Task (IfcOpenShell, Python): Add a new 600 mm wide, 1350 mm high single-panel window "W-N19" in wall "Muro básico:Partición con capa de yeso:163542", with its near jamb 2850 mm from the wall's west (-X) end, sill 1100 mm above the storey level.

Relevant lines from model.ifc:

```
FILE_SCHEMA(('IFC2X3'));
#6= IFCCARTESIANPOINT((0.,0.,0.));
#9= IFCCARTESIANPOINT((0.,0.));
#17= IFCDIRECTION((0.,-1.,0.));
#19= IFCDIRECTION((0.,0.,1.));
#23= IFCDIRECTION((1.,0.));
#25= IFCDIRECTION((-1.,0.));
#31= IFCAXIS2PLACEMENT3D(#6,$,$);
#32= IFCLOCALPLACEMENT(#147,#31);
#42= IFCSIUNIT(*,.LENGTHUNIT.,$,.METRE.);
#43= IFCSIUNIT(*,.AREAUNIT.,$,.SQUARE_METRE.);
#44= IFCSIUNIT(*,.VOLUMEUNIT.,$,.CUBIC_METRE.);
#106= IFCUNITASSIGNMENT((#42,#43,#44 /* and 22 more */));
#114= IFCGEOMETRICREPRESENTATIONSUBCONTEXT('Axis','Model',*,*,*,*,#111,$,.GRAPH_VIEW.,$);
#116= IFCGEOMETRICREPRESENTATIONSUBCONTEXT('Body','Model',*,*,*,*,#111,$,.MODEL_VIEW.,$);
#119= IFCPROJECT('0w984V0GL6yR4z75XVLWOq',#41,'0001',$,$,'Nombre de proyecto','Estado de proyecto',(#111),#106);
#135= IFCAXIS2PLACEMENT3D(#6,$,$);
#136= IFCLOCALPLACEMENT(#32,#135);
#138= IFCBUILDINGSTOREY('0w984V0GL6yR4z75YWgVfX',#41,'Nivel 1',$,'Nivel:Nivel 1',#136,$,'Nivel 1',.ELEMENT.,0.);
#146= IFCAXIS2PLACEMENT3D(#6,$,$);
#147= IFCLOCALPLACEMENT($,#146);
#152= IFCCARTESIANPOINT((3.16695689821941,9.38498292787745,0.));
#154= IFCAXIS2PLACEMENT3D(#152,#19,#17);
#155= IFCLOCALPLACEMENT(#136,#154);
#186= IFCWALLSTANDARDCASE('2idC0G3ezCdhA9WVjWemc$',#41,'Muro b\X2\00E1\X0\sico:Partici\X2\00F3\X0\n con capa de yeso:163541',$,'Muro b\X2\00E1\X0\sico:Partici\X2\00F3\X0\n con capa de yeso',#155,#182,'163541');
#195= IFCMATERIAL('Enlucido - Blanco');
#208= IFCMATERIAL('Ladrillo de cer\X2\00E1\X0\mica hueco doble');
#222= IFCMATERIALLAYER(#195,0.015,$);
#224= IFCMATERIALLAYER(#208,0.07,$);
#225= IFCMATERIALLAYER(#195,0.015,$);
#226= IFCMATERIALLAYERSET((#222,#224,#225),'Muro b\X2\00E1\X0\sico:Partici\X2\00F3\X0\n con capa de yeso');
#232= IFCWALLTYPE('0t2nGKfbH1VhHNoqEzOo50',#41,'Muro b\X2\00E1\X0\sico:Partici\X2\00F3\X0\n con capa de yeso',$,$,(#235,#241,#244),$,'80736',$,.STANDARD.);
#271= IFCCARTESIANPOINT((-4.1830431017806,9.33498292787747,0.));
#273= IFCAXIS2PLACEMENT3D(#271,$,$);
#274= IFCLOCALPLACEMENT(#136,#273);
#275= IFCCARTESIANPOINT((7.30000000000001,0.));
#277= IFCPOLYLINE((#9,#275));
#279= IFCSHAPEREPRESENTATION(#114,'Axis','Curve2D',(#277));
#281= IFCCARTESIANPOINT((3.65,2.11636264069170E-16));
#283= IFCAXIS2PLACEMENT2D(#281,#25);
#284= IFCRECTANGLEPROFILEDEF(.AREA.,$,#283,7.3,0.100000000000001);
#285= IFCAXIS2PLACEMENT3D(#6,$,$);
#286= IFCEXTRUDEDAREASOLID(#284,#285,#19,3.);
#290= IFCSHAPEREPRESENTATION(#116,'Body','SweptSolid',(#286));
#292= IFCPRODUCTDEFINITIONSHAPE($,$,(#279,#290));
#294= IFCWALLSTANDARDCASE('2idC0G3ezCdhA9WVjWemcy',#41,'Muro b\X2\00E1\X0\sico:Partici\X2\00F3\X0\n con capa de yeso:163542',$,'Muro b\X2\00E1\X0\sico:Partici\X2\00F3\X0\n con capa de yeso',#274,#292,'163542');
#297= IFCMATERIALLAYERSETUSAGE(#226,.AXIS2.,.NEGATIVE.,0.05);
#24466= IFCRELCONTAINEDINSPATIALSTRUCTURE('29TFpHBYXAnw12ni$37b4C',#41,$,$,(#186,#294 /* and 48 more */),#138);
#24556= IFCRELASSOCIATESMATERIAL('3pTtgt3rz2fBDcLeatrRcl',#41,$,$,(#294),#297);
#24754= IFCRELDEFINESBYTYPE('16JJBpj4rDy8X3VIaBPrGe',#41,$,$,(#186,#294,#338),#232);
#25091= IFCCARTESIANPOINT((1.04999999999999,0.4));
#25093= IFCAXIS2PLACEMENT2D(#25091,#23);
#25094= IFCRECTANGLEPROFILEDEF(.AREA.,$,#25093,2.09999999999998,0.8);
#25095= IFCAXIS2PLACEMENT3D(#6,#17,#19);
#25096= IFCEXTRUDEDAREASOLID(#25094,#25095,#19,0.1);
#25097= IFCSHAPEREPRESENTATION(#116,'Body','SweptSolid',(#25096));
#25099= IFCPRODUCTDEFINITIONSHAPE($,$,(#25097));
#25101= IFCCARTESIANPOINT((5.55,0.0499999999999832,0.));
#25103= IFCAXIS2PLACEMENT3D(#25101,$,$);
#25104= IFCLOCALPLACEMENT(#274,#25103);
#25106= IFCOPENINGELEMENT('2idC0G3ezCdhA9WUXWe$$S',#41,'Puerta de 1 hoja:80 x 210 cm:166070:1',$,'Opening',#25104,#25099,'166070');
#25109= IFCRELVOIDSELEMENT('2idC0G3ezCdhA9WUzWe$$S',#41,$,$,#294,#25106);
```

```python
import numpy as np
import ifcopenshell
import ifcopenshell.api.feature
import ifcopenshell.api.geometry
import ifcopenshell.api.root
import ifcopenshell.api.spatial
import ifcopenshell.api.type
import ifcopenshell.geom
import ifcopenshell.util.element
import ifcopenshell.util.placement
import ifcopenshell.util.representation
import ifcopenshell.util.shape
import ifcopenshell.util.unit

model = ifcopenshell.open("model.ifc")
unit_scale = ifcopenshell.util.unit.calculate_unit_scale(model)
settings = ifcopenshell.geom.settings()


def volume(element):
    """Net volume in cubic metres, openings subtracted."""
    shape = ifcopenshell.geom.create_shape(settings, element)
    return ifcopenshell.util.shape.get_volume(shape.geometry)


wall = model.by_id(294)
storey = ifcopenshell.util.element.get_container(wall, ifc_class="IfcBuildingStorey")
context = ifcopenshell.util.representation.get_context(model, "Model", "Body", "MODEL_VIEW")
before = volume(wall)

width, height, from_end, sill = 0.6, 1.35, 2.85, 1.1  # metres

# The wall runs along its own X axis, and the end named is its -X end.
wall_shape = ifcopenshell.geom.create_shape(settings, wall)
x, y, z = ifcopenshell.util.shape.get_vertices(wall_shape.geometry).T
start = x.min() + from_end
face, thickness = float(y.min()), float(y.max() - y.min())
wall_matrix = ifcopenshell.util.placement.get_local_placement(wall.ObjectPlacement)
level = ifcopenshell.util.placement.get_local_placement(storey.ObjectPlacement)[2, 3]


def in_wall(x, y):
    """Placement at x, y metres in the wall's axes, at sill height."""
    matrix = wall_matrix.copy()
    matrix[:, 3] = wall_matrix @ np.array([x / unit_scale, y / unit_scale, 0.0, 1.0])
    matrix[2, 3] = level + sill / unit_scale
    return matrix


# Opening: a box that overshoots both wall faces by 50 mm.
opening = ifcopenshell.api.root.create_entity(model, ifc_class="IfcOpeningElement")
box = ifcopenshell.api.geometry.add_wall_representation(
    model, context=context, length=width, height=height, thickness=thickness + 0.1
)
ifcopenshell.api.geometry.assign_representation(model, product=opening, representation=box)
ifcopenshell.api.geometry.edit_object_placement(model, product=opening, matrix=in_wall(start, face - 0.05), is_si=False)
ifcopenshell.api.feature.add_feature(model, feature=opening, element=wall)

window = ifcopenshell.api.root.create_entity(model, ifc_class="IfcWindow", name="W-N19")
window.OverallWidth, window.OverallHeight = width / unit_scale, height / unit_scale
body = ifcopenshell.api.geometry.add_window_representation(
    model,
    context=context,
    overall_width=window.OverallWidth,
    overall_height=window.OverallHeight,
    partition_type="SINGLE_PANEL",
)
ifcopenshell.api.geometry.assign_representation(model, product=window, representation=body)
ifcopenshell.api.spatial.assign_container(model, products=[window], relating_structure=storey)
fills = ifcopenshell.api.feature.add_filling(model, opening=opening, element=window)
fills.OwnerHistory = window.OwnerHistory  # required in IFC2X3

# IFC2X3 keeps the operation on the window style.
style = ifcopenshell.api.root.create_entity(model, ifc_class="IfcWindowStyle", name="W-N19")
style.OperationType, style.ConstructionType = "SINGLE_PANEL", "NOTDEFINED"
style.ParameterTakesPrecedence = style.Sizeable = False
ifcopenshell.api.type.assign_type(model, related_objects=[window], relating_type=style)

# Centre the window in the wall's thickness.
ifcopenshell.api.geometry.edit_object_placement(model, product=window, matrix=in_wall(start, face), is_si=False)
window_shape = ifcopenshell.geom.create_shape(settings, window)
depth = ifcopenshell.util.shape.get_vertices(window_shape.geometry)[:, 1]
offset = face + thickness / 2 - (depth.min() + depth.max()) / 2
ifcopenshell.api.geometry.edit_object_placement(model, product=window, matrix=in_wall(start, offset), is_si=False)

after = volume(wall)

print(f"wall volume {before:.3f} -> {after:.3f} m3")

model.write("model_v2.ifc")
```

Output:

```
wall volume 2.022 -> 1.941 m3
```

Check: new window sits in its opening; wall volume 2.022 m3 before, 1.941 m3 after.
